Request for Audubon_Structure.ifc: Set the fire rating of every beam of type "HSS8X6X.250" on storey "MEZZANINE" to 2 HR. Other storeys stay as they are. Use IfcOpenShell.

First a look at what the model holds.

```python
import ifcopenshell
import ifcopenshell.util.element

model = ifcopenshell.open("Audubon_Structure.ifc")
print(model.schema)
storey = next(s for s in model.by_type("IfcBuildingStorey") if s.Name == "MEZZANINE")
beams = [e for e in ifcopenshell.util.element.get_decomposition(storey) if e.is_a("IfcBeam")]
seen = {}
for e in beams:
    element_type = ifcopenshell.util.element.get_type(e)
    key = (element_type.Name if element_type != e and element_type else None, ifcopenshell.util.element.get_pset(e, "Pset_BeamCommon", "FireRating"))
    seen[key] = seen.get(key, 0) + 1
for (name, value), count in sorted(seen.items(), key=str):
    print(count, "x", name, "|", value)
```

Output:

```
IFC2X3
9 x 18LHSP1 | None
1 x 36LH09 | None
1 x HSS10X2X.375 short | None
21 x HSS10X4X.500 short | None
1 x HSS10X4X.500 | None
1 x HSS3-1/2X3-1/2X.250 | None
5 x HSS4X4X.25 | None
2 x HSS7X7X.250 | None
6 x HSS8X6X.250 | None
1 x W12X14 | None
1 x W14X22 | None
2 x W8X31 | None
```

```python
import ifcopenshell
import ifcopenshell.api.pset
import ifcopenshell.util.element

model = ifcopenshell.open("Audubon_Structure.ifc")

storey = next(s for s in model.by_type("IfcBuildingStorey") if s.Name == "MEZZANINE")
beams = [e for e in ifcopenshell.util.element.get_decomposition(storey) if e.is_a("IfcBeam")]

count = 0
for e in beams:
    element_type = ifcopenshell.util.element.get_type(e)
    if element_type in (None, e) or element_type.Name != "HSS8X6X.250":
        continue
    # add_pset returns the element's existing set when there is one.
    pset = ifcopenshell.api.pset.add_pset(model, product=e, name="Pset_BeamCommon")
    ifcopenshell.api.pset.edit_pset(model, pset=pset, properties={"FireRating": "2 HR"})
    count += 1

print(count, "beams updated")

model.write("Audubon_Structure_v2.ifc")
```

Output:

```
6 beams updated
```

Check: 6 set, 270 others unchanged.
